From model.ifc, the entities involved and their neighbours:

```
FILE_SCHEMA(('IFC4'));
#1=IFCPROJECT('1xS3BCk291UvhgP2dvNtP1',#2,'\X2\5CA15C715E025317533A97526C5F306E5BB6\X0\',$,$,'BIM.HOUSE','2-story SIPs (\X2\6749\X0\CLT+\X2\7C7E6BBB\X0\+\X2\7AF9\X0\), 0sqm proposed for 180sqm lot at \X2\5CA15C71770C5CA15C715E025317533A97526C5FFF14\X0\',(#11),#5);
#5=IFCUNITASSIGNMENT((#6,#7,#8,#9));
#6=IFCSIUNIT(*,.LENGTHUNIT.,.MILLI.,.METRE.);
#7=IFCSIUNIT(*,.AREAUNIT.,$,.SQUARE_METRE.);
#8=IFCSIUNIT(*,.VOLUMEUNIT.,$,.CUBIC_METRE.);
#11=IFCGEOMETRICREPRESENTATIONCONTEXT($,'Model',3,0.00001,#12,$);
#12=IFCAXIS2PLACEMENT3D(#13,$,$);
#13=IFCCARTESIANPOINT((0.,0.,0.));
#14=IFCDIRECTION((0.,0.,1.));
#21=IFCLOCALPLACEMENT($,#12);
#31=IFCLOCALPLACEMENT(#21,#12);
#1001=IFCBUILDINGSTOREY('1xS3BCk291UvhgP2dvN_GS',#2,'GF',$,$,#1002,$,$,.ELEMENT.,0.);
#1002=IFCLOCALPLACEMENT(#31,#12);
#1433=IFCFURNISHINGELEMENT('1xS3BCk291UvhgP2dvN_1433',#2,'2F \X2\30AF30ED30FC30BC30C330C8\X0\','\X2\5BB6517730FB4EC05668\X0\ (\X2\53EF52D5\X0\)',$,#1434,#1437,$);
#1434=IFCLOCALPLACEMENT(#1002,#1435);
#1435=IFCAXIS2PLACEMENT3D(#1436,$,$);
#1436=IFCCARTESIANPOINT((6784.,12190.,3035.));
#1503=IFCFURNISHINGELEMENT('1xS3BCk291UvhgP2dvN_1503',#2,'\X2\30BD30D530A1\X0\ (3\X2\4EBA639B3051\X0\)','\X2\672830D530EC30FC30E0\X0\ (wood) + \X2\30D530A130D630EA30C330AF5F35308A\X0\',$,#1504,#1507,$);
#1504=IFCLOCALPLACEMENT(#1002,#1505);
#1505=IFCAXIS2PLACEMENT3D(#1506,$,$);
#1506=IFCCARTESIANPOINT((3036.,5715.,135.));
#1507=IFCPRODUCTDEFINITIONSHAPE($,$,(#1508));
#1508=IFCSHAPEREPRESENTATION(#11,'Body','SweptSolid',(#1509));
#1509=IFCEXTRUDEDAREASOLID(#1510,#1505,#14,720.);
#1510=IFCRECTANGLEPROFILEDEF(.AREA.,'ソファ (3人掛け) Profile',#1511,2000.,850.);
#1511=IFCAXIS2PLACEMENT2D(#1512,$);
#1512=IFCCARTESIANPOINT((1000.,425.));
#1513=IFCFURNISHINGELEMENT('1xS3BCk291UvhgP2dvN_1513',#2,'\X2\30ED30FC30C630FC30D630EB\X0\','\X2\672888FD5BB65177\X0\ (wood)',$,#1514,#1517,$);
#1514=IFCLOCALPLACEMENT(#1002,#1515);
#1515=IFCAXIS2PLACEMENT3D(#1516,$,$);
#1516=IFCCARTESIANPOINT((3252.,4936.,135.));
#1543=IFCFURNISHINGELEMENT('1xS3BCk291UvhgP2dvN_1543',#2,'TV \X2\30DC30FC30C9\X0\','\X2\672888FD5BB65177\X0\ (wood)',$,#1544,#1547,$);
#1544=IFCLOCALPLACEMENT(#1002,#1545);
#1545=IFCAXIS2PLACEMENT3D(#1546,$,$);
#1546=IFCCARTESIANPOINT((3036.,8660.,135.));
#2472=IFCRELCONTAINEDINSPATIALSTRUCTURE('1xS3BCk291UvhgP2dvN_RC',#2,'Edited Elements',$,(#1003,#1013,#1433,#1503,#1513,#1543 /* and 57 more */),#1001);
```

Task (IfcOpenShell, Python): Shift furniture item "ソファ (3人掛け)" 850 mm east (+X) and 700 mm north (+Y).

```python
import ifcopenshell
import ifcopenshell.api.geometry
import ifcopenshell.util.placement

model = ifcopenshell.open("model.ifc")

item = model.by_guid("1xS3BCk291UvhgP2dvN_1503")
matrix = ifcopenshell.util.placement.get_local_placement(item.ObjectPlacement)
matrix[0, 3] += 850.0
matrix[1, 3] += 700.0
ifcopenshell.api.geometry.edit_object_placement(model, product=item, matrix=matrix, is_si=False)

print(ifcopenshell.util.placement.get_local_placement(item.ObjectPlacement).round(3) + 0.0)

model.write("model_v2.ifc")
```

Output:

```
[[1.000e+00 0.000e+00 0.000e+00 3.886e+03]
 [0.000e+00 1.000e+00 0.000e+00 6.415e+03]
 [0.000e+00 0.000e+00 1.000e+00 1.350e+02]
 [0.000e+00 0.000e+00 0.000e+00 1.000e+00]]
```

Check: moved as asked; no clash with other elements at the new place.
